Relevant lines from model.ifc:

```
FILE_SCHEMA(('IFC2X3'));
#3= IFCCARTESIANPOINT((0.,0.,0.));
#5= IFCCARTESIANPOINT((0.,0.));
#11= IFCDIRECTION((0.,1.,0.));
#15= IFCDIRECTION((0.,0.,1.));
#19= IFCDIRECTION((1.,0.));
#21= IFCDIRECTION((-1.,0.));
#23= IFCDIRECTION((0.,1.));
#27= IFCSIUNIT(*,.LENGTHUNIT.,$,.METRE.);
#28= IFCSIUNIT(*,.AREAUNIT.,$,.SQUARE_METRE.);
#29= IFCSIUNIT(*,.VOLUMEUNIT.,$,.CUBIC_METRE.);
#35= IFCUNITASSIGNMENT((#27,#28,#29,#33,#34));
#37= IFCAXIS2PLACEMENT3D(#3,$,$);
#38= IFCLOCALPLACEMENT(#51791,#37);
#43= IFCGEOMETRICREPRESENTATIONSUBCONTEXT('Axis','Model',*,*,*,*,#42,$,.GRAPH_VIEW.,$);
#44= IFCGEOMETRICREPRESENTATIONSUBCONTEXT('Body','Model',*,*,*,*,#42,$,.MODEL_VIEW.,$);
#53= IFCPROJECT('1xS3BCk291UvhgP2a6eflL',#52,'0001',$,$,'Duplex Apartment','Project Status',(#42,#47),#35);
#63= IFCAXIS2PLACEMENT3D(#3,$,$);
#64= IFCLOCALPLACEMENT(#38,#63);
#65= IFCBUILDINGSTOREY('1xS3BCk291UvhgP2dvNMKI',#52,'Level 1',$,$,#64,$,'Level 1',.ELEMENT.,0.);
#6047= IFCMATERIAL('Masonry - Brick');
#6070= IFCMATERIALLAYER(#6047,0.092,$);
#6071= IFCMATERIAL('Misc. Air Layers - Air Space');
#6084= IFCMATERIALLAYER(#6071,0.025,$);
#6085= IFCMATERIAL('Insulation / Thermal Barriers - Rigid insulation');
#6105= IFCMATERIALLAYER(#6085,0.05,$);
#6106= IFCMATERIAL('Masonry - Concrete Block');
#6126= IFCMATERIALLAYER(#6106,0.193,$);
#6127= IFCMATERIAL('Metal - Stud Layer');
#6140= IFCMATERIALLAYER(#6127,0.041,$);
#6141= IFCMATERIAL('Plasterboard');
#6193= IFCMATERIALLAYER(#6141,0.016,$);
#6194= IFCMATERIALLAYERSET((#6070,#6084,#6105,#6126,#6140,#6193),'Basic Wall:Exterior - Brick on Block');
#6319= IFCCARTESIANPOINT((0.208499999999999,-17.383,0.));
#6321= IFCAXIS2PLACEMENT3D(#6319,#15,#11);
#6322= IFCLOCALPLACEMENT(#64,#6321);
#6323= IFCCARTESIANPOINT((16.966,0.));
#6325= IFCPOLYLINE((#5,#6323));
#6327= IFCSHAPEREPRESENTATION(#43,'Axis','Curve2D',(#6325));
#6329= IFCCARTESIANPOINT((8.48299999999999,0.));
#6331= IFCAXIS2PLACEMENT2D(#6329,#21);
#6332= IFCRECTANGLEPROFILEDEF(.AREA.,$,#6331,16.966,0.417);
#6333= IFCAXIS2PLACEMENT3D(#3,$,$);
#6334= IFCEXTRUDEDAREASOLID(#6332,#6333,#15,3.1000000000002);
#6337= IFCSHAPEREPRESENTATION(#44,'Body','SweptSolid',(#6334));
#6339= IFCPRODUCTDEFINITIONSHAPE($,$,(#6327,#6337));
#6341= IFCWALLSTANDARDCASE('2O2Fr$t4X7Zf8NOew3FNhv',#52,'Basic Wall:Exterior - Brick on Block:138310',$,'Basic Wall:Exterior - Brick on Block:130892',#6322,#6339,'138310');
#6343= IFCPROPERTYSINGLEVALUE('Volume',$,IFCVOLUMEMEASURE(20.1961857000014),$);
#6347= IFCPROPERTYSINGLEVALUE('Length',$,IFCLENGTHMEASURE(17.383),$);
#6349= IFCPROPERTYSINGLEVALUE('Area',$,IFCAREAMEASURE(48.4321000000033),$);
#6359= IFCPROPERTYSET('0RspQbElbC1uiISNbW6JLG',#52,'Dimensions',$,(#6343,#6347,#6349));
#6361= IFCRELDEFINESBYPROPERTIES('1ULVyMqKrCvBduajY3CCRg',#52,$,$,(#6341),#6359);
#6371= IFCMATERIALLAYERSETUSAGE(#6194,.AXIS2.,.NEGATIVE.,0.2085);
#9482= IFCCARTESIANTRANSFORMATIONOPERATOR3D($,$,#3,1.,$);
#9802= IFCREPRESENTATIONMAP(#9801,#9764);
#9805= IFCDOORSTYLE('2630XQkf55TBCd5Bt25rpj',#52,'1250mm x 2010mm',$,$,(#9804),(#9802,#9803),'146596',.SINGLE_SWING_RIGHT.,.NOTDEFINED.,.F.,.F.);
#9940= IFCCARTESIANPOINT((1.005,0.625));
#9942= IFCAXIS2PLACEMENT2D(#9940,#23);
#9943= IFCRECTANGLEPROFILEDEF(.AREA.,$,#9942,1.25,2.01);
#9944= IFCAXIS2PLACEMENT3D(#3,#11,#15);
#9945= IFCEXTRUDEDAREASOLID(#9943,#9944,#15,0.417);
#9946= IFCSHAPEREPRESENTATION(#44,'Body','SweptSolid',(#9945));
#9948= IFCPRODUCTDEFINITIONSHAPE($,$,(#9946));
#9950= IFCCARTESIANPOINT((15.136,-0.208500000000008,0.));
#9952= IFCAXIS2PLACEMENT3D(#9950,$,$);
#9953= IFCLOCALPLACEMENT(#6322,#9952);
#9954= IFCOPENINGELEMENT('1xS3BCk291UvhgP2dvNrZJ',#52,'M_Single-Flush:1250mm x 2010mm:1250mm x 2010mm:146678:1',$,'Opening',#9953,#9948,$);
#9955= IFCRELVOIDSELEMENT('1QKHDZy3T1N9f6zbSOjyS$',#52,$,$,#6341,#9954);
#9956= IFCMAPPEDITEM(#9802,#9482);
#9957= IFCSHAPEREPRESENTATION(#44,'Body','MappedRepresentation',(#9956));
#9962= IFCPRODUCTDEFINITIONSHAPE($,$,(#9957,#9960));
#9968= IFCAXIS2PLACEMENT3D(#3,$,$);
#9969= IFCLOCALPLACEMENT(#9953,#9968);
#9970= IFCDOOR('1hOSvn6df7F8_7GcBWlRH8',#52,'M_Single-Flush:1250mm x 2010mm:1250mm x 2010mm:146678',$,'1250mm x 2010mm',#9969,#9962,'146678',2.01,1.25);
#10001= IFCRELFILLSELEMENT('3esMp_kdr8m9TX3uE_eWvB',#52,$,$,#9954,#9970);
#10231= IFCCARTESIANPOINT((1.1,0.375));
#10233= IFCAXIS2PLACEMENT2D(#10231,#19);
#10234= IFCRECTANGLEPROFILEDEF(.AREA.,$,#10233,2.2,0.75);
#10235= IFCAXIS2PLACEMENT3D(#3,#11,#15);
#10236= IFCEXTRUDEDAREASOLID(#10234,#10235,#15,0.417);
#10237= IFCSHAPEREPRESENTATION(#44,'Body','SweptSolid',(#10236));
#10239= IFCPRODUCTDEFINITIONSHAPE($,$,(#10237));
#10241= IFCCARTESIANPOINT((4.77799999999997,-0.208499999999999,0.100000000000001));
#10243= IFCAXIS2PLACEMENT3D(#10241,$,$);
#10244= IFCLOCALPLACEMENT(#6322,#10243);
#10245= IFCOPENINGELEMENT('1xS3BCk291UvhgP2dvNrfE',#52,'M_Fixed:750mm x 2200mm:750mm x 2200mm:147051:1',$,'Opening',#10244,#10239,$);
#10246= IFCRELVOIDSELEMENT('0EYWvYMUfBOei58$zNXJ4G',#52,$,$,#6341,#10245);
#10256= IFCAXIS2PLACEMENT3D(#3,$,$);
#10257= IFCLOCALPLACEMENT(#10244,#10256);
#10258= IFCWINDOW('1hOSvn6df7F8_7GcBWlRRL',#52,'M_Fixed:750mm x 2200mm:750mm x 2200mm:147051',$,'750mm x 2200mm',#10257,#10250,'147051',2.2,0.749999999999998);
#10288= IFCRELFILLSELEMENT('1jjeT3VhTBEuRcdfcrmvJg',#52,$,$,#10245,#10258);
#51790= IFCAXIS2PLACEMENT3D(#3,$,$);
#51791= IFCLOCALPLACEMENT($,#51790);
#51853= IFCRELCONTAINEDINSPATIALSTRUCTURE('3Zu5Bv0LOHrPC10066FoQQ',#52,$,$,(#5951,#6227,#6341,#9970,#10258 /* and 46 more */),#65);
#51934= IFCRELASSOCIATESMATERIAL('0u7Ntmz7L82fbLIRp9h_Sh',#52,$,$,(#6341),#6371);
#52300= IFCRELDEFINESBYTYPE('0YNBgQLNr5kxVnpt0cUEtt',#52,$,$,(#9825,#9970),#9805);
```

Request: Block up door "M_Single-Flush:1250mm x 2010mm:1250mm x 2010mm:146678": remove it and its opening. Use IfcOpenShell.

```python
import ifcopenshell
import ifcopenshell.api.feature
import ifcopenshell.api.pset
import ifcopenshell.api.root
import ifcopenshell.geom
import ifcopenshell.util.element
import ifcopenshell.util.shape
import ifcopenshell.util.unit

model = ifcopenshell.open("model.ifc")
area_scale = ifcopenshell.util.unit.calculate_unit_scale(model, "AREAUNIT")
volume_scale = ifcopenshell.util.unit.calculate_unit_scale(model, "VOLUMEUNIT")
settings = ifcopenshell.geom.settings()


def volume(element):
    """Net volume in cubic metres, openings subtracted."""
    shape = ifcopenshell.geom.create_shape(settings, element)
    return ifcopenshell.util.shape.get_volume(shape.geometry)


door = model.by_guid("1hOSvn6df7F8_7GcBWlRH8")
opening = door.FillsVoids[0].RelatingOpeningElement
wall = opening.VoidsElements[0].RelatingBuildingElement
before = volume(wall)

ifcopenshell.api.root.remove_product(model, product=door)
ifcopenshell.api.feature.remove_feature(model, feature=opening)

after = volume(wall)
thickness = 0.417  # wall thickness in metres

# Update the wall's stored quantities.
pset = model.by_id(ifcopenshell.util.element.get_pset(wall, "Dimensions", should_inherit=False)["id"])
ifcopenshell.api.pset.edit_pset(model, pset=pset, properties={
    "Volume": model.create_entity("IfcVolumeMeasure", after / volume_scale),
    "Area": model.create_entity("IfcAreaMeasure", after / thickness / area_scale),
})

print(f"wall volume {before:.3f} -> {after:.3f} m3")

model.write("model_v2.ifc")
```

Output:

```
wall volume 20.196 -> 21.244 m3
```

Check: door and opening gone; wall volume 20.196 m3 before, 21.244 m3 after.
